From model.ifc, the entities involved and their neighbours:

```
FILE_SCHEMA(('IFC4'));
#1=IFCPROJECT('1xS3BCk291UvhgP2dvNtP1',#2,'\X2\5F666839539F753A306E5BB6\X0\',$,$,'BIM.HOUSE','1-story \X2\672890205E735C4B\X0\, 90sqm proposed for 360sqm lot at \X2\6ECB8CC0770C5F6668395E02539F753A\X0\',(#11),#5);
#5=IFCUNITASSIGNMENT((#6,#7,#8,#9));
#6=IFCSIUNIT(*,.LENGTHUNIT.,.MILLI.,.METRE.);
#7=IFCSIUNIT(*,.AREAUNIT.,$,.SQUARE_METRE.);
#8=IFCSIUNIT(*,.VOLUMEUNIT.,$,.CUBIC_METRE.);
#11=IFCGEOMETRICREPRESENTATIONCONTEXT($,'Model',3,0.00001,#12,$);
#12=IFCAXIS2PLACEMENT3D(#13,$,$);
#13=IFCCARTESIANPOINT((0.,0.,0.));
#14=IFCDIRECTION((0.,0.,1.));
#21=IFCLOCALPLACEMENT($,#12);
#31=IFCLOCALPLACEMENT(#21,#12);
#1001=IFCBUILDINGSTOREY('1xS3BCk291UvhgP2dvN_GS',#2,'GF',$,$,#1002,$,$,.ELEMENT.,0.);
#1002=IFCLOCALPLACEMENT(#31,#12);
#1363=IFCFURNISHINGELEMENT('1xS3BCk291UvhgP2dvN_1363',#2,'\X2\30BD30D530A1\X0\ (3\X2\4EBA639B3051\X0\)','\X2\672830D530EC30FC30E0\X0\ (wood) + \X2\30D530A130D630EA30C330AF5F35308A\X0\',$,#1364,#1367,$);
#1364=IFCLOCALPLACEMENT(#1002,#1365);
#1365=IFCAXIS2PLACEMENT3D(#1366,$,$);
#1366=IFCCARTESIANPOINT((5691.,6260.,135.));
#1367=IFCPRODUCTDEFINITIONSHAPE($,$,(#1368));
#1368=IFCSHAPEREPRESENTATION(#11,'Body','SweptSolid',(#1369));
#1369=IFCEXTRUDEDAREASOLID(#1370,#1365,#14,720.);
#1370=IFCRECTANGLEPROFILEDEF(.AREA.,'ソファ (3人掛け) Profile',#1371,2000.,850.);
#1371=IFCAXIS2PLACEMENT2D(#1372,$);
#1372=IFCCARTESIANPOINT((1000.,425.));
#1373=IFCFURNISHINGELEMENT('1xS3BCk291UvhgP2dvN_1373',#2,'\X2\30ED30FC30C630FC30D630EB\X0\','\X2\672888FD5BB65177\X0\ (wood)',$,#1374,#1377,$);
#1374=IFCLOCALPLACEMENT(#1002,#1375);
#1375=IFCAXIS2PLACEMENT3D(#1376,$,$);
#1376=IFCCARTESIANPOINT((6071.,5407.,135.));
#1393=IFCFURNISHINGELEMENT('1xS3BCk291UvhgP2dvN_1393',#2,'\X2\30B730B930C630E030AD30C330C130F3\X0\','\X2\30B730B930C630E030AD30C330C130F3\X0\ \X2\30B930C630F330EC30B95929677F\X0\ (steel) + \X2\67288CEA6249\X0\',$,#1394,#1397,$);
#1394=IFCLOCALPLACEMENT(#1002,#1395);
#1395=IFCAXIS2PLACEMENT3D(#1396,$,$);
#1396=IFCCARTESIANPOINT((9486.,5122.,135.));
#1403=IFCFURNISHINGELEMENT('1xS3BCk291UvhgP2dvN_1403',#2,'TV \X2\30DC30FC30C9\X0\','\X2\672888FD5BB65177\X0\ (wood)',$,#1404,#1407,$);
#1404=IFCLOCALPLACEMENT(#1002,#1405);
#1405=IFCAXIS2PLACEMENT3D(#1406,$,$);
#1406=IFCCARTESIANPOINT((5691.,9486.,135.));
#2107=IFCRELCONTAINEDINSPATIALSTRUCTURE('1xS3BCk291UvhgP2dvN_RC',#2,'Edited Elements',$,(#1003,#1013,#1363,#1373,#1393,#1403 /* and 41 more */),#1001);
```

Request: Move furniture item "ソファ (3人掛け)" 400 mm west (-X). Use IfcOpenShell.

```python
import ifcopenshell
import ifcopenshell.api.geometry
import ifcopenshell.util.placement
import ifcopenshell.util.unit

model = ifcopenshell.open("model.ifc")
unit_scale = ifcopenshell.util.unit.calculate_unit_scale(model)

item = model.by_guid("1xS3BCk291UvhgP2dvN_1363")
matrix = ifcopenshell.util.placement.get_local_placement(item.ObjectPlacement)
matrix[0, 3] -= 0.4 / unit_scale
ifcopenshell.api.geometry.edit_object_placement(model, product=item, matrix=matrix, is_si=False)

print(ifcopenshell.util.placement.get_local_placement(item.ObjectPlacement).round(3) + 0.0)

model.write("model_v2.ifc")
```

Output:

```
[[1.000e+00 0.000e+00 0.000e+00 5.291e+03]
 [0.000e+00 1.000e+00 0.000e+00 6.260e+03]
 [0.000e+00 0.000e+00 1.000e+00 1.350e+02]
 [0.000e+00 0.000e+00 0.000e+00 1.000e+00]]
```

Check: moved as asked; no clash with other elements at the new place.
